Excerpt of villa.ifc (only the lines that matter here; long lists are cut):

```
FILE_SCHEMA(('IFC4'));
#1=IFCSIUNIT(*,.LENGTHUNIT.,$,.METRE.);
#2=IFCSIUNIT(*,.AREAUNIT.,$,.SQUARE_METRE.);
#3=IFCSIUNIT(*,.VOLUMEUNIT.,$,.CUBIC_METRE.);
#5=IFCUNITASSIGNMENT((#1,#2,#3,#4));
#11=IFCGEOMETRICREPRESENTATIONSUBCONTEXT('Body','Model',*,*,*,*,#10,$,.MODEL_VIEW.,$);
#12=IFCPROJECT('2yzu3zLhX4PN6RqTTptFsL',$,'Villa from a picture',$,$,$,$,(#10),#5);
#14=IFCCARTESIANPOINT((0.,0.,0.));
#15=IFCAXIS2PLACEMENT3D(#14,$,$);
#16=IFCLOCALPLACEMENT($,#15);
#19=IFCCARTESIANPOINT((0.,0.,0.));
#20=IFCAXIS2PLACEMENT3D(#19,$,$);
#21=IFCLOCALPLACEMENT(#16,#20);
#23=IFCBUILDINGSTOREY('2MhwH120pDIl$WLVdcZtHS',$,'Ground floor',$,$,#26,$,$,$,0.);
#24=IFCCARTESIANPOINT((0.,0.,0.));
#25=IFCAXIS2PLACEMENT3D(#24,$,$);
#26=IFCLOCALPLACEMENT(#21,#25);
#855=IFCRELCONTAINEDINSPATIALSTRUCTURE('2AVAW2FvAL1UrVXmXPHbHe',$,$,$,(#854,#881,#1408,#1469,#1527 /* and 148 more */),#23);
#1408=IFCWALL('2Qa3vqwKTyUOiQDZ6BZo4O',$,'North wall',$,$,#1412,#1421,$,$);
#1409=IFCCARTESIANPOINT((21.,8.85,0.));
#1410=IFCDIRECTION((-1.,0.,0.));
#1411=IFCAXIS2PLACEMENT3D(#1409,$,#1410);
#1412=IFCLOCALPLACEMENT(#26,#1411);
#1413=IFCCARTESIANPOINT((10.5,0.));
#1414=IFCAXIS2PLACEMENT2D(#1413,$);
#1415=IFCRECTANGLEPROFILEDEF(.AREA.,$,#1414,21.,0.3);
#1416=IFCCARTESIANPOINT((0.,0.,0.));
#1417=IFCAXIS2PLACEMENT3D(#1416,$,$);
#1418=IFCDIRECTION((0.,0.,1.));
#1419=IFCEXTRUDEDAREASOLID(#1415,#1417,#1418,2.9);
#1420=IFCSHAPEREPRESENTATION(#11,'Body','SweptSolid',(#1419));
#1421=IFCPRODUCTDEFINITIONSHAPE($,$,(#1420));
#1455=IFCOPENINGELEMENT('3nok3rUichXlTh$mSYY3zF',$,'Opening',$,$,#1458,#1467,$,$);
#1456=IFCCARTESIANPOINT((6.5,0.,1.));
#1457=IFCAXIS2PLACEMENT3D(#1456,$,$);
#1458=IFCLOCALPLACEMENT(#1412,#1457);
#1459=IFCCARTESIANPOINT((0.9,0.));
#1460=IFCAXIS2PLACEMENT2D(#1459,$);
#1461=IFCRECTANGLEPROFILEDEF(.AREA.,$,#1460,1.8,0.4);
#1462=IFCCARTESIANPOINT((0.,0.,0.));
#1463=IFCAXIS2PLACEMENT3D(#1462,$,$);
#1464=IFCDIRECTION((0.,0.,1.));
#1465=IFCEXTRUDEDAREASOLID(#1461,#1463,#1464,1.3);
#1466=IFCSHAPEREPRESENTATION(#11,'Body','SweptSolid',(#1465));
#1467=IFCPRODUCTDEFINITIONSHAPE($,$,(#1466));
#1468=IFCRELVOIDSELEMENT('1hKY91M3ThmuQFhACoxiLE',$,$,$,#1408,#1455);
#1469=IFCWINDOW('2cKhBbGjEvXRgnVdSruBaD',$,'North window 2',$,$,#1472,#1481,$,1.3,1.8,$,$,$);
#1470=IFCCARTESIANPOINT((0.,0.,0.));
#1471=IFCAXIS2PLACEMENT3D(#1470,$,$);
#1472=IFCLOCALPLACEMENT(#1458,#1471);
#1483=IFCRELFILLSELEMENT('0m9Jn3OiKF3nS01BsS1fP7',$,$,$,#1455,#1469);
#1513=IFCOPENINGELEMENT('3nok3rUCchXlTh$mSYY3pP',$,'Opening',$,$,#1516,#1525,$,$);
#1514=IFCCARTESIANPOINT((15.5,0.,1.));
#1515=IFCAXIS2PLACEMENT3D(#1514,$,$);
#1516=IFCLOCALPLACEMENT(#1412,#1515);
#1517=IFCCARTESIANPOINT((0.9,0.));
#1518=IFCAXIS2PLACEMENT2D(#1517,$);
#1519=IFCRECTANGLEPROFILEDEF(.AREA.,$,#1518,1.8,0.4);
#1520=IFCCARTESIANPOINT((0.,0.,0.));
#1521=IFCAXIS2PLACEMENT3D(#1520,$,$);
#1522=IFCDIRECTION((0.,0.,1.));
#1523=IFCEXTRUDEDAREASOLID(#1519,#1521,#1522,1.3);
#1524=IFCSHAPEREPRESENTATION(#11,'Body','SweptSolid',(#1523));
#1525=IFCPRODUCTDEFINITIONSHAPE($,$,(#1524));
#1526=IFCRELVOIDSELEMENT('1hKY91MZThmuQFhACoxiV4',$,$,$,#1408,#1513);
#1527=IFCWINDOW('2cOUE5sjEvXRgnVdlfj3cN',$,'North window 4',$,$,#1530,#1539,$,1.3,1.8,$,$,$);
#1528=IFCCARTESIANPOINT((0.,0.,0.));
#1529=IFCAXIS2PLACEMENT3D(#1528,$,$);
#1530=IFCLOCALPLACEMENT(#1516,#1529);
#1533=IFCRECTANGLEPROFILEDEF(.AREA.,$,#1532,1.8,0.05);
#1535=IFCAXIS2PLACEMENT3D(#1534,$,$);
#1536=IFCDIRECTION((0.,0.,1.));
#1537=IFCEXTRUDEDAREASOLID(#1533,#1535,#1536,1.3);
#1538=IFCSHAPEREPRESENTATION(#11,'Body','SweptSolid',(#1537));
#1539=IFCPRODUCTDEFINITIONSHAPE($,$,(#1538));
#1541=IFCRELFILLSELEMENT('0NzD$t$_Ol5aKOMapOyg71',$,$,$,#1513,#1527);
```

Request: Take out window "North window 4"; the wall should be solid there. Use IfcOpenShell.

```python
import ifcopenshell
import ifcopenshell.api.feature
import ifcopenshell.api.root
import ifcopenshell.geom
import ifcopenshell.util.shape

model = ifcopenshell.open("villa.ifc")
settings = ifcopenshell.geom.settings()


def volume(element):
    """Net volume in cubic metres, openings subtracted."""
    shape = ifcopenshell.geom.create_shape(settings, element)
    return ifcopenshell.util.shape.get_volume(shape.geometry)


window = model.by_guid("2cOUE5sjEvXRgnVdlfj3cN")
opening = window.FillsVoids[0].RelatingOpeningElement
wall = opening.VoidsElements[0].RelatingBuildingElement
before = volume(wall)

ifcopenshell.api.root.remove_product(model, product=window)
ifcopenshell.api.feature.remove_feature(model, feature=opening)

after = volume(wall)

print(f"wall volume {before:.3f} -> {after:.3f} m3")

model.write("villa_edited.ifc")
```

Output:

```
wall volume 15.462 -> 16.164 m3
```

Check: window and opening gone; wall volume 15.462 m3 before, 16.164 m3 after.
